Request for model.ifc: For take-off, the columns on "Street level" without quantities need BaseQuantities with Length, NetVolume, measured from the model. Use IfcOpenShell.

First a look at what the model holds.

```python
import ifcopenshell
import ifcopenshell.util.element
import ifcopenshell.util.unit

model = ifcopenshell.open("model.ifc")
print(model.schema)
for unit_type in ("LENGTHUNIT", "AREAUNIT", "VOLUMEUNIT"):
    print(unit_type, ifcopenshell.util.unit.calculate_unit_scale(model, unit_type))
storey = next(s for s in model.by_type("IfcBuildingStorey") if s.Name == "Street level")
columns = [e for e in ifcopenshell.util.element.get_decomposition(storey) if e.is_a("IfcColumn")]
for e in sorted(columns, key=lambda e: e.id()):
    print(e.id(), e.is_a(), e.Name, list(ifcopenshell.util.element.get_psets(e, qtos_only=True)), sep=" | ")
```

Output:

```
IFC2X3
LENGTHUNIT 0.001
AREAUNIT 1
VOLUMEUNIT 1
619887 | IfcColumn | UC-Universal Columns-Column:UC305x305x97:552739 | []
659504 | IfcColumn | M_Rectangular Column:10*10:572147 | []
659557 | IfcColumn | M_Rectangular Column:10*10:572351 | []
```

```python
import ifcopenshell
import ifcopenshell.api.pset
import ifcopenshell.geom
import ifcopenshell.util.element
import ifcopenshell.util.shape
import ifcopenshell.util.unit

model = ifcopenshell.open("model.ifc")
unit_scale = ifcopenshell.util.unit.calculate_unit_scale(model)
volume_scale = ifcopenshell.util.unit.calculate_unit_scale(model, "VOLUMEUNIT")
settings = ifcopenshell.geom.settings()

storey = next(s for s in model.by_type("IfcBuildingStorey") if s.Name == "Street level")
columns = [e for e in ifcopenshell.util.element.get_decomposition(storey) if e.is_a("IfcColumn")]

for e in sorted(columns, key=lambda e: e.id()):
    if ifcopenshell.util.element.get_psets(e, qtos_only=True, should_inherit=False):
        continue
    # Geometry comes back in metres, in the element's own axes.
    shape = ifcopenshell.geom.create_shape(settings, e)
    values = {
        "Length": ifcopenshell.util.shape.get_z(shape.geometry) / unit_scale,
        "NetVolume": ifcopenshell.util.shape.get_volume(shape.geometry) / volume_scale,
    }
    qto = ifcopenshell.api.pset.add_qto(model, product=e, name="BaseQuantities")
    ifcopenshell.api.pset.edit_qto(model, qto=qto, properties=values)
    print(e.id(), {k: round(v, 3) for k, v in values.items()})

model.write("model_v2.ifc")
```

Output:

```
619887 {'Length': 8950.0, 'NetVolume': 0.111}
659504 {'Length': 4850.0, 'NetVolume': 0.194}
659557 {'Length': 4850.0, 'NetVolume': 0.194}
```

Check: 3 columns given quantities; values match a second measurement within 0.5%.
